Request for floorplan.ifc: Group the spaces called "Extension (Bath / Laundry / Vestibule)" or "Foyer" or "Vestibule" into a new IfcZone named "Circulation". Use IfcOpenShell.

First a look at what the model holds.

```python
import ifcopenshell

model = ifcopenshell.open("floorplan.ifc")
print(model.schema)
seen = {}
for space in model.by_type("IfcSpace"):
    seen[space.LongName] = seen.get(space.LongName, 0) + 1
for name, count in sorted(seen.items(), key=str):
    print(count, "x", name)
print("zones:", [z.Name for z in model.by_type("IfcZone")][:20])
```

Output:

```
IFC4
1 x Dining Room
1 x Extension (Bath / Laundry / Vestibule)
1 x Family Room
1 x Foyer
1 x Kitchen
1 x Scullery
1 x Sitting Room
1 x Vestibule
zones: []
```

```python
import ifcopenshell
import ifcopenshell.api.group
import ifcopenshell.api.root

model = ifcopenshell.open("floorplan.ifc")

names = {"Extension (Bath / Laundry / Vestibule)", "Foyer", "Vestibule"}
spaces = [s for s in model.by_type("IfcSpace") if s.LongName in names]

zone = ifcopenshell.api.root.create_entity(model, ifc_class="IfcZone", name="Circulation")
ifcopenshell.api.group.assign_group(model, products=spaces, group=zone)
print(len(spaces), "spaces in", zone.Name)

model.write("floorplan_edited.ifc")
```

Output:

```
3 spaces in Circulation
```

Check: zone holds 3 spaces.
